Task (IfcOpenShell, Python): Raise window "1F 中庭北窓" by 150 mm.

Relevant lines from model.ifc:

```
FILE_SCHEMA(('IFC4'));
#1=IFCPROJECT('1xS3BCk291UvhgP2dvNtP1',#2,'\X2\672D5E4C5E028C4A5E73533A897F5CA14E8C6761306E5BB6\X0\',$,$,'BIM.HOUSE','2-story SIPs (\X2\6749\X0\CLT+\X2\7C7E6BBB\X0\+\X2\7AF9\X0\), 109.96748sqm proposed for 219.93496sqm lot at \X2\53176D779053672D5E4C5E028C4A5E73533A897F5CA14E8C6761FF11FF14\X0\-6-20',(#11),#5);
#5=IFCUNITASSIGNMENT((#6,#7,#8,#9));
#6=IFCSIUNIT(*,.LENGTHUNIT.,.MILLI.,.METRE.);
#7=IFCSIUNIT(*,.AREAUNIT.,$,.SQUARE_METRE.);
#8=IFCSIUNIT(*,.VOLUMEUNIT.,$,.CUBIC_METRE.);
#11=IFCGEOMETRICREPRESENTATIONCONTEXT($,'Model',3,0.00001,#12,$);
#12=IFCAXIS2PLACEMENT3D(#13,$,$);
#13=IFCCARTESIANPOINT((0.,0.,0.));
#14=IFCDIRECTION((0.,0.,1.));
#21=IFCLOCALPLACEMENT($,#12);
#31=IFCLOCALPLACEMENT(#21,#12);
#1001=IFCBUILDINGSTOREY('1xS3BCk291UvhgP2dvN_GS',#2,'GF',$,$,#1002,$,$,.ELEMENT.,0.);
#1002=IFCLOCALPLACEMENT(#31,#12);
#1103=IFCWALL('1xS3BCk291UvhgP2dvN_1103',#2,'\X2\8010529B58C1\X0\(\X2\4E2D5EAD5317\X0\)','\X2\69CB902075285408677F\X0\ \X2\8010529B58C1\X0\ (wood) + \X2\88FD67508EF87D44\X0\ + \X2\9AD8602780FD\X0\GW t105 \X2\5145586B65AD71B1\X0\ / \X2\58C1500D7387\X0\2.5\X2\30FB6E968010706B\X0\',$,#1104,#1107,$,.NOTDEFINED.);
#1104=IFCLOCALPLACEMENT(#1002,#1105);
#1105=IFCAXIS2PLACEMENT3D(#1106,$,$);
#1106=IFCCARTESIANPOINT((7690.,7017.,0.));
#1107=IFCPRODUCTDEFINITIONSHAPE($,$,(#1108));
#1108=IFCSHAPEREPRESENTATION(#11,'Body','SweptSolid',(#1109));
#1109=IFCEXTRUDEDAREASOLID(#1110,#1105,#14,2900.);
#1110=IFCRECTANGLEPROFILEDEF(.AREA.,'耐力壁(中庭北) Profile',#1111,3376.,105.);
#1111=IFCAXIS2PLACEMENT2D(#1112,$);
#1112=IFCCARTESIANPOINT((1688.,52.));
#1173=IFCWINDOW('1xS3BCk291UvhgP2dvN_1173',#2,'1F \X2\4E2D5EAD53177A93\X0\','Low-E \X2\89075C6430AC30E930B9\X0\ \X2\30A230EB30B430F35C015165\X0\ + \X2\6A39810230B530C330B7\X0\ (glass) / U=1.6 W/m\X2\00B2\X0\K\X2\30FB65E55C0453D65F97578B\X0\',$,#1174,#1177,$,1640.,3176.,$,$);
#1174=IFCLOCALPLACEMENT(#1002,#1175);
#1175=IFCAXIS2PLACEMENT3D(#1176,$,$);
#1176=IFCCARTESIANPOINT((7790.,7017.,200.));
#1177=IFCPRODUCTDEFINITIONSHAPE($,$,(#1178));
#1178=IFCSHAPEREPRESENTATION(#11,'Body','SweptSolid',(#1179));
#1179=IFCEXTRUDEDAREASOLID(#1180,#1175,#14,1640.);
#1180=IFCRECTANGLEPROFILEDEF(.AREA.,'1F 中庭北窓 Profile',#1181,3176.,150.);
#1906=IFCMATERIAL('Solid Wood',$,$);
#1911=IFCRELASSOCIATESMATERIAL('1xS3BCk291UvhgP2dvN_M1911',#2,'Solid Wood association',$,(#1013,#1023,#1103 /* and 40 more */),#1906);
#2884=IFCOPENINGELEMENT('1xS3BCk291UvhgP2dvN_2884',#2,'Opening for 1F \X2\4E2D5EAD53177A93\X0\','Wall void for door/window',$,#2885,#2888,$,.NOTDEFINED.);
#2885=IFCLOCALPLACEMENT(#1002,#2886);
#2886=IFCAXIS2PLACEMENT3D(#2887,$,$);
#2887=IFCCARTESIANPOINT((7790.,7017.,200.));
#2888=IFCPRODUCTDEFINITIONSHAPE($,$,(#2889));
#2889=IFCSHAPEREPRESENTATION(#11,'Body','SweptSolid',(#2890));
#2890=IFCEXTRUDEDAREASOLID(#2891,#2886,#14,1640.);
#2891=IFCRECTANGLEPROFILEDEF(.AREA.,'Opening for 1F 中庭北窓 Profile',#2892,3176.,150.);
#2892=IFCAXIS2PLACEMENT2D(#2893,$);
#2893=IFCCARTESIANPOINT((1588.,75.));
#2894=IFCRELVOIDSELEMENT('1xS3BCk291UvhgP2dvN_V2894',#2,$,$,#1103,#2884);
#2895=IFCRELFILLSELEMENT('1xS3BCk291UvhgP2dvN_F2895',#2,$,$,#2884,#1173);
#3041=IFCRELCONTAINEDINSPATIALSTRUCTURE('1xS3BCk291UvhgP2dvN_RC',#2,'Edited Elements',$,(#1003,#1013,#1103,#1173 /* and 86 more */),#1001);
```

```python
import numpy as np
import ifcopenshell
import ifcopenshell.api.geometry
import ifcopenshell.util.placement
import ifcopenshell.util.unit

model = ifcopenshell.open("model.ifc")
unit_scale = ifcopenshell.util.unit.calculate_unit_scale(model)

window = model.by_guid("1xS3BCk291UvhgP2dvN_1173")
opening = window.FillsVoids[0].RelatingOpeningElement
dz = 0.15 / unit_scale

shift = np.array([0.0, 0.0, dz])
# The window is not placed relative to its opening, so move both.
for product in (opening, window):
    matrix = ifcopenshell.util.placement.get_local_placement(product.ObjectPlacement)
    matrix[:3, 3] += shift
    ifcopenshell.api.geometry.edit_object_placement(model, product=product, matrix=matrix, is_si=False)

print(f"moved by {dz * unit_scale:+.3f} m")

model.write("model_v2.ifc")
```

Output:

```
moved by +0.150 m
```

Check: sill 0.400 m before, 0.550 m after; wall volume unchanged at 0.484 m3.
